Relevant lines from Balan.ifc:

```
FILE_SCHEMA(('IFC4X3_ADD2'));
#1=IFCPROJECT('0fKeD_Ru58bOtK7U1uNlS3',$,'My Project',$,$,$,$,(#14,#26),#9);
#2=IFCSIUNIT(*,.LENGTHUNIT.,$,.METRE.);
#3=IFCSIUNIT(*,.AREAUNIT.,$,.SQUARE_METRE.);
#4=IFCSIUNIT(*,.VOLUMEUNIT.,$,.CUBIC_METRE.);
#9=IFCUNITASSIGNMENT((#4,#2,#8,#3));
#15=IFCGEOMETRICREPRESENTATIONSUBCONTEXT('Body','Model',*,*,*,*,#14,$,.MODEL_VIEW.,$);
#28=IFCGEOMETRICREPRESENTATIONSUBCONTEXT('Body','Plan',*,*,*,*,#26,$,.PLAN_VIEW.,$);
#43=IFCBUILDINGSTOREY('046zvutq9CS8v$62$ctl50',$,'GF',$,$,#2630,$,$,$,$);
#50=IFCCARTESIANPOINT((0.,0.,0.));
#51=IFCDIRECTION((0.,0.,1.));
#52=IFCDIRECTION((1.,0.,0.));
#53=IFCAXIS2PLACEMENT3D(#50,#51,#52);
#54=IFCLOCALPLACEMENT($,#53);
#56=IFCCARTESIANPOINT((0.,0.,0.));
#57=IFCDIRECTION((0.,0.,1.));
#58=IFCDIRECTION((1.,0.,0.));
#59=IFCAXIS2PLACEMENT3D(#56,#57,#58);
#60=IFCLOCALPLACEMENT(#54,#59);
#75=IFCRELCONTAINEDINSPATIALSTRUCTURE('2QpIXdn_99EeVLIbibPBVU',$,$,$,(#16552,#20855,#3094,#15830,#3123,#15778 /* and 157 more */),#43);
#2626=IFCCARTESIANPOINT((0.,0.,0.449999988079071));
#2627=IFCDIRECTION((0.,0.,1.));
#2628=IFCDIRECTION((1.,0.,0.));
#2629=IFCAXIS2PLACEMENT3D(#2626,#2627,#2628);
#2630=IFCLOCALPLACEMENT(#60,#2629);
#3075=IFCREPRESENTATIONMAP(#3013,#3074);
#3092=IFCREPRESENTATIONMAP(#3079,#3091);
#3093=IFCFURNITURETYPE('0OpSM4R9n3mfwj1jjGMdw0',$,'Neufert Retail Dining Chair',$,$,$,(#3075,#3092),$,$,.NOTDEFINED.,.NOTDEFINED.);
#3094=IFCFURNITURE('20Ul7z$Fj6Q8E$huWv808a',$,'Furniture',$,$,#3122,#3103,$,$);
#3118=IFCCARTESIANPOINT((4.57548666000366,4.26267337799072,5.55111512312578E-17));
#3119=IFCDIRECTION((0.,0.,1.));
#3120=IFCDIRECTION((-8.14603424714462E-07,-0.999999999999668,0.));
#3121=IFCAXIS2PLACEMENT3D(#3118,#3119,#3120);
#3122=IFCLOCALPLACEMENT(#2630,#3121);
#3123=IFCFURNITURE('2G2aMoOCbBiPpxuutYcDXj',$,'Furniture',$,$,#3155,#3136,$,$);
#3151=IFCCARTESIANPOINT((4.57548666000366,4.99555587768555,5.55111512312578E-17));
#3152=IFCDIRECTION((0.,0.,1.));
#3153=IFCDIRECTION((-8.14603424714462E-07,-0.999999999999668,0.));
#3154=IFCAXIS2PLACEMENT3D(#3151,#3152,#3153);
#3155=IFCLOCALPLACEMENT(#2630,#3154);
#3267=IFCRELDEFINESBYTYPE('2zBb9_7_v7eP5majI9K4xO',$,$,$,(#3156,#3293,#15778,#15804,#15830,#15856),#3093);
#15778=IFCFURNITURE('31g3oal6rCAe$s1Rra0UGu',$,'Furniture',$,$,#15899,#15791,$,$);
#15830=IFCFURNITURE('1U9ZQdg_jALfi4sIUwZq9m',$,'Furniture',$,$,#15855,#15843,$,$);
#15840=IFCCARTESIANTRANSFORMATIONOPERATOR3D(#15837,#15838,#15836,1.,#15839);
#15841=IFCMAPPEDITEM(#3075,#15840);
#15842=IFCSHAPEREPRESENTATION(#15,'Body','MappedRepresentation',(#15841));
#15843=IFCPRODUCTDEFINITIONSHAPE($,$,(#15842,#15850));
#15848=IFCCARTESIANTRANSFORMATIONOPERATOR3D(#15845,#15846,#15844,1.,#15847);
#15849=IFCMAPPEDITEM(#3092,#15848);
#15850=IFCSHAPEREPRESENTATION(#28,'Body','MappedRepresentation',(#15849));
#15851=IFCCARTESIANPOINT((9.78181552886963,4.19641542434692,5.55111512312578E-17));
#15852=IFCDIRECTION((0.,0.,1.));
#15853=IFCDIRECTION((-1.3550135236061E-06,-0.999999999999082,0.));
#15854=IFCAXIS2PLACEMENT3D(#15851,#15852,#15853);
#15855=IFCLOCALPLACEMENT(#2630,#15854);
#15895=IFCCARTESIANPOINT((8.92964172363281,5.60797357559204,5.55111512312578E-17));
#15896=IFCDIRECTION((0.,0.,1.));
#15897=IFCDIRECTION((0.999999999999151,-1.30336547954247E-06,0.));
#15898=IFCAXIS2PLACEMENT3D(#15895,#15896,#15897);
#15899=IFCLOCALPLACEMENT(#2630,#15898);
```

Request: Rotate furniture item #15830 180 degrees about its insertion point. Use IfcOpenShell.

```python
import ifcopenshell
import ifcopenshell.api.geometry
import ifcopenshell.util.placement

model = ifcopenshell.open("Balan.ifc")

item = model.by_id(15830)
matrix = ifcopenshell.util.placement.get_local_placement(item.ObjectPlacement)
matrix = matrix @ ifcopenshell.util.placement.rotation(180, "Z")
ifcopenshell.api.geometry.edit_object_placement(model, product=item, matrix=matrix, is_si=False)

print(ifcopenshell.util.placement.get_local_placement(item.ObjectPlacement).round(3) + 0.0)

model.write("Balan_v2.ifc")
```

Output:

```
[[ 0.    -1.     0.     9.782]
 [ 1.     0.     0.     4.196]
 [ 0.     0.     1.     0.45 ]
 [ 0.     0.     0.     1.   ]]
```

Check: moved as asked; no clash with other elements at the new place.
